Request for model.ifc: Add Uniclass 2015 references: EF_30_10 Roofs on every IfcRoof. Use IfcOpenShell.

First a look at what the model holds.

```python
import ifcopenshell

model = ifcopenshell.open("model.ifc")
print(model.schema)
print("classifications:", [c.Name for c in model.by_type("IfcClassification")])
for ifc_class in ("IfcDoor", "IfcRoof", "IfcStair", "IfcWall", "IfcWindow"):
    print(ifc_class, len(model.by_type(ifc_class)))
```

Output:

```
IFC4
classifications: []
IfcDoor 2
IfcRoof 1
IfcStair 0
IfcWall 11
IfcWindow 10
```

```python
import ifcopenshell
import ifcopenshell.api.classification

model = ifcopenshell.open("model.ifc")

system = ifcopenshell.api.classification.add_classification(model, classification="Uniclass 2015")

codes = {
    "IfcRoof": ("EF_30_10", "Roofs"),
}
for ifc_class, (code, name) in codes.items():
    products = model.by_type(ifc_class)
    ifcopenshell.api.classification.add_reference(
        model, products=products, classification=system, identification=code, name=name
    )
    print(code, len(products))

model.write("model_v2.ifc")
```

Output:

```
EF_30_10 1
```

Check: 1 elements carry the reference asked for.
